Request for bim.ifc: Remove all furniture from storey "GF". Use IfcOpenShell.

First a look at what the model holds.

```python
import ifcopenshell
import ifcopenshell.util.element

model = ifcopenshell.open("bim.ifc")
print(model.schema)
storey = next(s for s in model.by_type("IfcBuildingStorey") if s.Name == "GF")
furniture = [e for e in ifcopenshell.util.element.get_decomposition(storey) if e.is_a("IfcFurnishingElement")]
seen = {}
for e in furniture:
    element_type = ifcopenshell.util.element.get_type(e)
    name = element_type.Name if element_type not in (None, e) else None
    seen[name] = seen.get(name, 0) + 1
for name, count in sorted(seen.items(), key=str):
    print(count, "x", name)
```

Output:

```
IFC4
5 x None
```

```python
import ifcopenshell
import ifcopenshell.api.root
import ifcopenshell.util.element

model = ifcopenshell.open("bim.ifc")

storey = next(s for s in model.by_type("IfcBuildingStorey") if s.Name == "GF")
furniture = [e for e in ifcopenshell.util.element.get_decomposition(storey) if e.is_a("IfcFurnishingElement")]

for e in furniture:
    ifcopenshell.api.root.remove_product(model, product=e)
print(len(furniture), "removed")

model.write("bim-out.ifc")
```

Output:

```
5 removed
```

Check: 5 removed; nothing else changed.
